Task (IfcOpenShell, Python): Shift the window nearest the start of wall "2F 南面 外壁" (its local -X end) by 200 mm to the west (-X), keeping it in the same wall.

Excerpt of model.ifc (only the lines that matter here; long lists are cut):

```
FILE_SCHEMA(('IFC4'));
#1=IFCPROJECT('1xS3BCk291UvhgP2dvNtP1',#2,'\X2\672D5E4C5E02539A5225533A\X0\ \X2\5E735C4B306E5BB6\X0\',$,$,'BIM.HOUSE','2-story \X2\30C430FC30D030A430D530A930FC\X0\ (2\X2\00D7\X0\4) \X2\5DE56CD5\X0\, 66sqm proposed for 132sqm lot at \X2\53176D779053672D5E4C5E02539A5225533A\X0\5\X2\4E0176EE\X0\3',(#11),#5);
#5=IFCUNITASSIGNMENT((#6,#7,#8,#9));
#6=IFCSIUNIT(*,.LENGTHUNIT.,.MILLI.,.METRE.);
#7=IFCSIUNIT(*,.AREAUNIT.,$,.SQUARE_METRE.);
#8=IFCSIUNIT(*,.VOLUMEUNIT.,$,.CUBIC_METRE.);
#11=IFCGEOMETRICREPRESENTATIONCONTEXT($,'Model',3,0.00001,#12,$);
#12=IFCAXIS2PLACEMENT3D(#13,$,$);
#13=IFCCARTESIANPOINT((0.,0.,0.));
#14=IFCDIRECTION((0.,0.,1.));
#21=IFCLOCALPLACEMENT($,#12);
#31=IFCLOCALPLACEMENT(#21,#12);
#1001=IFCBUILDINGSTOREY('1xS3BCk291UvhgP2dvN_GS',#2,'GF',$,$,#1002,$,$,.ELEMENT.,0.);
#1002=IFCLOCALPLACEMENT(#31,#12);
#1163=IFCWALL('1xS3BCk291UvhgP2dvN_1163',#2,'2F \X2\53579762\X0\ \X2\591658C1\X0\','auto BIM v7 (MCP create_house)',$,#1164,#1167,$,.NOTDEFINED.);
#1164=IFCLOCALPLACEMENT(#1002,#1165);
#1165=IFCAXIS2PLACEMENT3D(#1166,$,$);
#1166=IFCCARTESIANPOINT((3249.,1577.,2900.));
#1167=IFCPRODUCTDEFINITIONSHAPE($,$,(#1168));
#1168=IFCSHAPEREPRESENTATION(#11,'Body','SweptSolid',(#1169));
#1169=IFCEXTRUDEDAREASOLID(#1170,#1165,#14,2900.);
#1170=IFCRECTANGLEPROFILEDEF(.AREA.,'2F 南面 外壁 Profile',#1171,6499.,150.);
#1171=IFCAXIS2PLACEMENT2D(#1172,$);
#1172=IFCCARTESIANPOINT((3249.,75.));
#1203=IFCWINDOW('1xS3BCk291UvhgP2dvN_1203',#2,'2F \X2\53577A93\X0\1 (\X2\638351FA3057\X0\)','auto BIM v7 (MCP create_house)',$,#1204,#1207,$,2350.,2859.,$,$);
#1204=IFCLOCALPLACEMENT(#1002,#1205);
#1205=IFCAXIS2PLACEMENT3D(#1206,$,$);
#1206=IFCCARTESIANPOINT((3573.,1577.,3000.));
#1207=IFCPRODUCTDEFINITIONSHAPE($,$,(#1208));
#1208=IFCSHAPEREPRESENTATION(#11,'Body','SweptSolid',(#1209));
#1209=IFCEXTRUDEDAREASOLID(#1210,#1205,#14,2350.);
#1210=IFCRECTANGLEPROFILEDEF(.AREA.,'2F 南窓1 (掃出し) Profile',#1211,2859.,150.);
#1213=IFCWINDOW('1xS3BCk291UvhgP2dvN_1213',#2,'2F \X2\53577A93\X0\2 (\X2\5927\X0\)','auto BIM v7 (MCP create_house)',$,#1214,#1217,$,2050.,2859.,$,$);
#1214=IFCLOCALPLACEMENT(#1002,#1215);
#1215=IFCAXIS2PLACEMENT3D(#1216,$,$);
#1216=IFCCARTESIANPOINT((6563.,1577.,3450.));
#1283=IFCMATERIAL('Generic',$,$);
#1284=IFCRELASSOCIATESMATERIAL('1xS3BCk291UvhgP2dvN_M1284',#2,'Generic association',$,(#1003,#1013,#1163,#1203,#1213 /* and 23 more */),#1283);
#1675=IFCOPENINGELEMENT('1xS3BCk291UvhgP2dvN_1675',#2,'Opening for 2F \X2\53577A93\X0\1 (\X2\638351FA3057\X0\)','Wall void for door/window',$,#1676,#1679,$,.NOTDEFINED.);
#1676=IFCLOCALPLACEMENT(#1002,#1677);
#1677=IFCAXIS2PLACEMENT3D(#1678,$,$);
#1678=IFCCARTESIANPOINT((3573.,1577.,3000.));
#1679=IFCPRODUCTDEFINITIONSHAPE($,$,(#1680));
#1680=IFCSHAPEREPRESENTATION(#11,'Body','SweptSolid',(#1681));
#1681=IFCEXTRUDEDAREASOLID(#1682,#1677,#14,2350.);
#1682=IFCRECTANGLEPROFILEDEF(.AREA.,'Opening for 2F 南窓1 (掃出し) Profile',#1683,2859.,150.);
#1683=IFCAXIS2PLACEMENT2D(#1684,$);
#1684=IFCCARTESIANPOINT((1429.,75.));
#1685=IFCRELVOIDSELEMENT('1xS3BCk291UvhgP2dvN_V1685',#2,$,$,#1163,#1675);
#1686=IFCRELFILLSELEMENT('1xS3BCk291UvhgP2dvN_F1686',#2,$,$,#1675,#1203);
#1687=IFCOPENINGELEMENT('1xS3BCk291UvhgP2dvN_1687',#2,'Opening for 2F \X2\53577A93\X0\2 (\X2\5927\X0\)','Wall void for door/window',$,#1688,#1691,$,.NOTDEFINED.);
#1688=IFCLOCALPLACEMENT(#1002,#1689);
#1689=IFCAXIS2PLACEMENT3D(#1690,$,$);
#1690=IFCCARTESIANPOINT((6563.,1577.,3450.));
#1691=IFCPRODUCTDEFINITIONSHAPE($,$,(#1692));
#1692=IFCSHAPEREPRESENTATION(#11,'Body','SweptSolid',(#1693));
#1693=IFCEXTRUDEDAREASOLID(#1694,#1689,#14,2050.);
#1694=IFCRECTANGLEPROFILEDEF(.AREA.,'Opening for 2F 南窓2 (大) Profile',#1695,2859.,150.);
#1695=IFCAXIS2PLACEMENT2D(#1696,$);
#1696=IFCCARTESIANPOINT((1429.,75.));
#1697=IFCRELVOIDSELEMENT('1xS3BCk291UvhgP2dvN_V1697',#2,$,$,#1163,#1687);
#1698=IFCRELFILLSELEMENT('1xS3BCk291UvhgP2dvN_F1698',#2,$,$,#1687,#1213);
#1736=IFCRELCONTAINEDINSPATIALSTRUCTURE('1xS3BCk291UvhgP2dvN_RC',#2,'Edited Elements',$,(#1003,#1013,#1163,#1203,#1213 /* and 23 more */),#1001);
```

```python
import ifcopenshell
import ifcopenshell.api.geometry
import ifcopenshell.util.placement

model = ifcopenshell.open("model.ifc")

window = model.by_guid("1xS3BCk291UvhgP2dvN_1203")
opening = window.FillsVoids[0].RelatingOpeningElement
wall = opening.VoidsElements[0].RelatingBuildingElement

wall_matrix = ifcopenshell.util.placement.get_local_placement(wall.ObjectPlacement)
shift = wall_matrix[:3, 0] * -200.0
before = ifcopenshell.util.placement.get_local_placement(window.ObjectPlacement)[:3, 3].copy()

# The window is not placed relative to its opening, so move both.
for product in (opening, window):
    matrix = ifcopenshell.util.placement.get_local_placement(product.ObjectPlacement)
    matrix[:3, 3] += shift
    ifcopenshell.api.geometry.edit_object_placement(model, product=product, matrix=matrix, is_si=False)

after = ifcopenshell.util.placement.get_local_placement(window.ObjectPlacement)[:3, 3]
print("window moved by", (after - before).round(3) + 0.0)

model.write("model_edited.ifc")
```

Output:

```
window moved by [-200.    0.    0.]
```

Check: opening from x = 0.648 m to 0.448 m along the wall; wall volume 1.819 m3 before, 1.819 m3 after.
